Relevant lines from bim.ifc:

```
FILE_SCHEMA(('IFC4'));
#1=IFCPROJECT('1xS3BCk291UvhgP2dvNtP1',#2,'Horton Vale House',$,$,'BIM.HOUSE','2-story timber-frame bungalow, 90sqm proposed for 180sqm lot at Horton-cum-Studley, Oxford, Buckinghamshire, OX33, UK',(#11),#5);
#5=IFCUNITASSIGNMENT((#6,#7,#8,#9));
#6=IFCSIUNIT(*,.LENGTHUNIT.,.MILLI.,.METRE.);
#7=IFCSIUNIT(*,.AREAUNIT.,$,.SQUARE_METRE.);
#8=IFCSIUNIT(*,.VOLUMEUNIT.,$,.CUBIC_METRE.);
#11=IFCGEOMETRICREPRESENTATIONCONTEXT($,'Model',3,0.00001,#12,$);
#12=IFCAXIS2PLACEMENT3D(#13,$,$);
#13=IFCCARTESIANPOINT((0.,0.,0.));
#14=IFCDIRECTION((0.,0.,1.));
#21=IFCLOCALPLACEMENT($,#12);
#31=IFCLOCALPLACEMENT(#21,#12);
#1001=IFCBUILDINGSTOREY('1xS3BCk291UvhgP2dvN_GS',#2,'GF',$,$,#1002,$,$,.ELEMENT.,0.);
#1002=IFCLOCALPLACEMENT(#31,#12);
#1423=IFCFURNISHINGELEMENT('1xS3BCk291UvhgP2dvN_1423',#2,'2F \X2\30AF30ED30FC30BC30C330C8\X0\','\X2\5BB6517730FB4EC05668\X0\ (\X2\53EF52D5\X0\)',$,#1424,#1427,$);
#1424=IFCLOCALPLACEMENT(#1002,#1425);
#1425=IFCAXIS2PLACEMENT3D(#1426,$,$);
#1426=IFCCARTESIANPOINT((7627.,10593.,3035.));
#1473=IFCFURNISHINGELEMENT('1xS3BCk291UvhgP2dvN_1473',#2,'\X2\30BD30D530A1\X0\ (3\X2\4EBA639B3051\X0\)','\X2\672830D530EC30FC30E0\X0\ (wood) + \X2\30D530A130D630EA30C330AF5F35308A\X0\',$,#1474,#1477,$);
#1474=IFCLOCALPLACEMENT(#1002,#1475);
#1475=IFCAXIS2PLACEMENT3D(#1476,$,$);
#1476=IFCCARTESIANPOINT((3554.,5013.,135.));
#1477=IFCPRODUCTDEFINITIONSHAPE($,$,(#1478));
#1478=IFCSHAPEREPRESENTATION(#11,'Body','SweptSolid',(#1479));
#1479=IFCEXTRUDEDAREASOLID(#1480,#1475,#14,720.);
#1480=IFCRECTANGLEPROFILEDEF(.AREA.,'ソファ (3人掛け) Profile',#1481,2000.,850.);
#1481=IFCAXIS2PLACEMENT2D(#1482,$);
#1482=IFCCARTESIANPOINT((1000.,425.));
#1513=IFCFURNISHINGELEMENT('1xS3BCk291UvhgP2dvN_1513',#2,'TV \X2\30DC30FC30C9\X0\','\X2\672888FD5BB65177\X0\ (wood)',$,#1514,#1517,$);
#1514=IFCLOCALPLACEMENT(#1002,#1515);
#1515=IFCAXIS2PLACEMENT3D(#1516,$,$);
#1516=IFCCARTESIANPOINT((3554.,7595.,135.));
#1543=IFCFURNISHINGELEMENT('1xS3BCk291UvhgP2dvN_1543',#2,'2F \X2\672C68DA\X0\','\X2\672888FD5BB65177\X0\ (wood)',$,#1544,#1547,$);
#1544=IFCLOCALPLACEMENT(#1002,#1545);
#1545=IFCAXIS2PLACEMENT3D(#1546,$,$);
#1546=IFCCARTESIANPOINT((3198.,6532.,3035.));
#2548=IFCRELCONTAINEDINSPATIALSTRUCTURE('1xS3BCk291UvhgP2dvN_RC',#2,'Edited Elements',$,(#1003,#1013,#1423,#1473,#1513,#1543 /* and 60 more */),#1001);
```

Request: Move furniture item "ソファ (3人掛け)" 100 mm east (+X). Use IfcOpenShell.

```python
import ifcopenshell
import ifcopenshell.api.geometry
import ifcopenshell.util.placement
import ifcopenshell.util.unit

model = ifcopenshell.open("bim.ifc")
unit_scale = ifcopenshell.util.unit.calculate_unit_scale(model)

item = model.by_guid("1xS3BCk291UvhgP2dvN_1473")
matrix = ifcopenshell.util.placement.get_local_placement(item.ObjectPlacement)
matrix[0, 3] += 0.1 / unit_scale
ifcopenshell.api.geometry.edit_object_placement(model, product=item, matrix=matrix, is_si=False)

print(ifcopenshell.util.placement.get_local_placement(item.ObjectPlacement).round(3) + 0.0)

model.write("bim_rev.ifc")
```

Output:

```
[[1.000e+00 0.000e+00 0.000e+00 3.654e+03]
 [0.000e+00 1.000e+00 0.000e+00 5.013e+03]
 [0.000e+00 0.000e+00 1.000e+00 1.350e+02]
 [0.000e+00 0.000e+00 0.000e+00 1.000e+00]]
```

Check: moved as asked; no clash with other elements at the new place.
